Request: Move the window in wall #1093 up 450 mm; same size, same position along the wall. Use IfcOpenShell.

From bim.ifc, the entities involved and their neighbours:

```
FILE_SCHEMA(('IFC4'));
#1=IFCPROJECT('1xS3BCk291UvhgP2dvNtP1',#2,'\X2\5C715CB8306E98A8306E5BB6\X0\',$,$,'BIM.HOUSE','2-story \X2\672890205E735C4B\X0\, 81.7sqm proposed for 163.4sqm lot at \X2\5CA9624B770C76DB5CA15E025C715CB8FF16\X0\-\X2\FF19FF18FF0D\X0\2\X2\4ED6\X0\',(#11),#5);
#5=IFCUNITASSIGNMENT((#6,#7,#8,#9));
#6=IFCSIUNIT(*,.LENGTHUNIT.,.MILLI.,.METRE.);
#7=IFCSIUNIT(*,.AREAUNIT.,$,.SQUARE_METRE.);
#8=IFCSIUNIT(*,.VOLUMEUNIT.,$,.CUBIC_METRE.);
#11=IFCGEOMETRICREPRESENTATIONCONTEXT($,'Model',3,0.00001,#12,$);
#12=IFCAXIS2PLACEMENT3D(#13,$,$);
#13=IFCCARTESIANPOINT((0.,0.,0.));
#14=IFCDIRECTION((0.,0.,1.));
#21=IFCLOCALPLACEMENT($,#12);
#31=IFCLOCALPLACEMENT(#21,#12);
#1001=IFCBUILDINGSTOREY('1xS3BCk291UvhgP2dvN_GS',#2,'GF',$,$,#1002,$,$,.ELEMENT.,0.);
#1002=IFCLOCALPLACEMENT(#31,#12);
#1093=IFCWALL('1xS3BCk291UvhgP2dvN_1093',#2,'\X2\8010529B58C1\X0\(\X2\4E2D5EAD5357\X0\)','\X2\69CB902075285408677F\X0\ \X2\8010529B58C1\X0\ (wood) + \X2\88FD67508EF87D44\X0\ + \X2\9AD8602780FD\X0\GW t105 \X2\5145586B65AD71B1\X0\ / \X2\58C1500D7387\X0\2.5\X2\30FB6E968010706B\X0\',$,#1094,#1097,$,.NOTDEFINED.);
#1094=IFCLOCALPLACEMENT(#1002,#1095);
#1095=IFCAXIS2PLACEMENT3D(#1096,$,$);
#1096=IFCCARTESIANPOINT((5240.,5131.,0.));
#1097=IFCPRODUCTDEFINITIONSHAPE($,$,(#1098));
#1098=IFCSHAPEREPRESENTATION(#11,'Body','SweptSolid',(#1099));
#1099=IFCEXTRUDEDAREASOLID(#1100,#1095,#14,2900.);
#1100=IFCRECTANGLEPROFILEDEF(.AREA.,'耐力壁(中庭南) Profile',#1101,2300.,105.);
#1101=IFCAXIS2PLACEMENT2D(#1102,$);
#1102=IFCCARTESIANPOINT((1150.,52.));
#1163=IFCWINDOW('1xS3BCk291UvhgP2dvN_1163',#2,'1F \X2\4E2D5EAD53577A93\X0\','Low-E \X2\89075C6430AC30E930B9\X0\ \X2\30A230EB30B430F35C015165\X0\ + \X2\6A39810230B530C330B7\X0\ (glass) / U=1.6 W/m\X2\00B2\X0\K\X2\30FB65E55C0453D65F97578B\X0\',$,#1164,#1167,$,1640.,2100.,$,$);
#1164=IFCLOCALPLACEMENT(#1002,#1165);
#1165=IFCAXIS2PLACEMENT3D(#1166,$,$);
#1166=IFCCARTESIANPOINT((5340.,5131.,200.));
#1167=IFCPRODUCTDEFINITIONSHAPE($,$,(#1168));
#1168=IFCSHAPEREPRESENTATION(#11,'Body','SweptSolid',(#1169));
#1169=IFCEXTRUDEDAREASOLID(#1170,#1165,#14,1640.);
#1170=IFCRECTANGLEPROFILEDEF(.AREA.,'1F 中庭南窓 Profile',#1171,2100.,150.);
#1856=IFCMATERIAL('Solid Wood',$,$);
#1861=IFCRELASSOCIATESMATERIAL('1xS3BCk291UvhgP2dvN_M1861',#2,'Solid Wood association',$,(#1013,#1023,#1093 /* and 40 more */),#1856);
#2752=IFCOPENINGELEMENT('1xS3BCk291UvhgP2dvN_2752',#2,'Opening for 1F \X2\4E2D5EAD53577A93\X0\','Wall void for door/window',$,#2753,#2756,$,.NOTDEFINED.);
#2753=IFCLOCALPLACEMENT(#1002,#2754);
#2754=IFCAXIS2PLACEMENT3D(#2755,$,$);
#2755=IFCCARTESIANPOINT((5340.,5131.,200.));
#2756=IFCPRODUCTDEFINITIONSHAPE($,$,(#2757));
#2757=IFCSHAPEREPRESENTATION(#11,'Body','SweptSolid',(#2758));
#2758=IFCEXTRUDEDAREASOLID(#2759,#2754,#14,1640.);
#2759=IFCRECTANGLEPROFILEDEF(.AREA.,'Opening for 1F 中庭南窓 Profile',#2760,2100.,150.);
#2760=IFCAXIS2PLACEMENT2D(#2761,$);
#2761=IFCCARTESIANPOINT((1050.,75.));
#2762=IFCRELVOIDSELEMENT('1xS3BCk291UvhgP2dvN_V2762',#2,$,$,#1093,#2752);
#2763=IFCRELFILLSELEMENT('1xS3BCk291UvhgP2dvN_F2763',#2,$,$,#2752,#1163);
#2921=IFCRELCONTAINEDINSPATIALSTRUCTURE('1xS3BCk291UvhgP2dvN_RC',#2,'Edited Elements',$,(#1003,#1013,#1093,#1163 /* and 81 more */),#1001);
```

```python
import numpy as np
import ifcopenshell
import ifcopenshell.api.geometry
import ifcopenshell.util.placement
import ifcopenshell.util.unit

model = ifcopenshell.open("bim.ifc")
unit_scale = ifcopenshell.util.unit.calculate_unit_scale(model)

window = model.by_guid("1xS3BCk291UvhgP2dvN_1163")
opening = window.FillsVoids[0].RelatingOpeningElement
dz = 450.0

shift = np.array([0.0, 0.0, dz])
# The window is not placed relative to its opening, so move both.
for product in (opening, window):
    matrix = ifcopenshell.util.placement.get_local_placement(product.ObjectPlacement)
    matrix[:3, 3] += shift
    ifcopenshell.api.geometry.edit_object_placement(model, product=product, matrix=matrix, is_si=False)

print(f"moved by {dz * unit_scale:+.3f} m")

model.write("bim-out.ifc")
```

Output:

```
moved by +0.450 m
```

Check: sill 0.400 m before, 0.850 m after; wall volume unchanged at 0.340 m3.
